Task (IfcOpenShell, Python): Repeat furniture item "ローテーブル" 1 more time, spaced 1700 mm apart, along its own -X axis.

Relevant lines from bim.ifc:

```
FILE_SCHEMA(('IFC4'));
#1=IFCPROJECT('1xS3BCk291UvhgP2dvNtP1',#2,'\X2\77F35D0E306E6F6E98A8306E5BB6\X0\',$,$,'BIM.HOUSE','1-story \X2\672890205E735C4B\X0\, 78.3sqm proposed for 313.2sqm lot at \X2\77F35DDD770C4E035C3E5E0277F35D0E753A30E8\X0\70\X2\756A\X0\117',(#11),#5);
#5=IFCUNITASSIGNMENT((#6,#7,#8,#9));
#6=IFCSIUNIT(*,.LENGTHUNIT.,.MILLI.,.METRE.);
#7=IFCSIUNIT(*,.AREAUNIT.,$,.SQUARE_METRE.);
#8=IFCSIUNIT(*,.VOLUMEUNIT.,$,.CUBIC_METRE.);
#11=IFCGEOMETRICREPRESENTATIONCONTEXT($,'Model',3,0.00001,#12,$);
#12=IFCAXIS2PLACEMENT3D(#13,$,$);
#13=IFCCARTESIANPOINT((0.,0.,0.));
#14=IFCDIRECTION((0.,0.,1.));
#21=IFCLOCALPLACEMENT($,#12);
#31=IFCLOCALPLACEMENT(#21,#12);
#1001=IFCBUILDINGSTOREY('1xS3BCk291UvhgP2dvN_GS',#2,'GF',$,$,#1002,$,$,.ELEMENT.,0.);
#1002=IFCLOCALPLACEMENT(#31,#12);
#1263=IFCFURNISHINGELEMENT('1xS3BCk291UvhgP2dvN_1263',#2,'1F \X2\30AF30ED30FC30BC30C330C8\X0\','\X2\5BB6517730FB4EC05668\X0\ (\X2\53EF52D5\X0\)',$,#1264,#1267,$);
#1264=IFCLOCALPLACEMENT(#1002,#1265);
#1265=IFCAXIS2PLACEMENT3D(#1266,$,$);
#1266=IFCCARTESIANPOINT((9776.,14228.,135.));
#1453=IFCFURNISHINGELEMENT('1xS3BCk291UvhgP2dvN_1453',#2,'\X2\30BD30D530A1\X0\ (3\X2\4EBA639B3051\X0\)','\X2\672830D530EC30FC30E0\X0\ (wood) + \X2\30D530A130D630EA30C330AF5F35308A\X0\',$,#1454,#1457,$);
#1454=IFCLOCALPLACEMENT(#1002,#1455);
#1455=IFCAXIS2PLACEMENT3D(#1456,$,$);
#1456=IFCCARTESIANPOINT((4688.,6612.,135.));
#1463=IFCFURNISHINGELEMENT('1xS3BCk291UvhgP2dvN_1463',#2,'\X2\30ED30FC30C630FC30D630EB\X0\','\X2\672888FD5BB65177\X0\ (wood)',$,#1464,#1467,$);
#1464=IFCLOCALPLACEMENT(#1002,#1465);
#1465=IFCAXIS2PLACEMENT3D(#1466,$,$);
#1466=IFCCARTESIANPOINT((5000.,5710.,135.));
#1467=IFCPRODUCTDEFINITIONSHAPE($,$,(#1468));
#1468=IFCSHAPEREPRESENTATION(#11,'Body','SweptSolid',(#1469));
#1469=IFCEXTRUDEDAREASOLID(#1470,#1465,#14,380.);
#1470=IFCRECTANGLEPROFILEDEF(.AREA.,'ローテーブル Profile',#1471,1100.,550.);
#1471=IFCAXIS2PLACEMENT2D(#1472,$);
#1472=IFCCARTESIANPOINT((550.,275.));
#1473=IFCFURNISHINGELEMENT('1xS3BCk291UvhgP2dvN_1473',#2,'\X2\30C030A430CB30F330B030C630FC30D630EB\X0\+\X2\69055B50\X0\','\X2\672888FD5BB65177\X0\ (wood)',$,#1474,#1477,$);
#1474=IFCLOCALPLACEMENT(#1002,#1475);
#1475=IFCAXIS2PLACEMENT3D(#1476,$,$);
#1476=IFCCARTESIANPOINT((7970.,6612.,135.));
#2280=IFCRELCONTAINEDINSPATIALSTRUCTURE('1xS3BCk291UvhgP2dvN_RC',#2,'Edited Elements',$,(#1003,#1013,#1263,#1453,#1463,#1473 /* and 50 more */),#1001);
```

```python
import ifcopenshell
import ifcopenshell.api.geometry
import ifcopenshell.api.root
import ifcopenshell.util.element
import ifcopenshell.util.placement
import ifcopenshell.util.unit

model = ifcopenshell.open("bim.ifc")
unit_scale = ifcopenshell.util.unit.calculate_unit_scale(model)


def reuse_history(source, copy):
    """copy_class also copies each property set's owner history, people and application; keep the originals."""
    for rel in copy.IsDefinedBy:
        if rel.is_a("IfcRelDefinesByProperties") and (history := rel.RelatingPropertyDefinition.OwnerHistory):
            rel.RelatingPropertyDefinition.OwnerHistory = source.OwnerHistory
            ifcopenshell.util.element.remove_deep2(model, history)


source = model.by_guid("1xS3BCk291UvhgP2dvN_1463")
base = ifcopenshell.util.placement.get_local_placement(source.ObjectPlacement)
step = -base[:3, 0] * 1.7 / unit_scale

for i in range(1, 2):
    copy = ifcopenshell.api.root.copy_class(model, product=source)
    copy.Representation = ifcopenshell.util.element.copy_deep(
        model, source.Representation, exclude=["IfcGeometricRepresentationContext", "IfcRepresentationMap"]
    )
    reuse_history(source, copy)
    matrix = base.copy()
    matrix[:3, 3] += i * step
    print("added at", matrix[:3, 3].round(3) + 0.0)
    ifcopenshell.api.geometry.edit_object_placement(model, product=copy, matrix=matrix, is_si=False)

model.write("bim_rev.ifc")
```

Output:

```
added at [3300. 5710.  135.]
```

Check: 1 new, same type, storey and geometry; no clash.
